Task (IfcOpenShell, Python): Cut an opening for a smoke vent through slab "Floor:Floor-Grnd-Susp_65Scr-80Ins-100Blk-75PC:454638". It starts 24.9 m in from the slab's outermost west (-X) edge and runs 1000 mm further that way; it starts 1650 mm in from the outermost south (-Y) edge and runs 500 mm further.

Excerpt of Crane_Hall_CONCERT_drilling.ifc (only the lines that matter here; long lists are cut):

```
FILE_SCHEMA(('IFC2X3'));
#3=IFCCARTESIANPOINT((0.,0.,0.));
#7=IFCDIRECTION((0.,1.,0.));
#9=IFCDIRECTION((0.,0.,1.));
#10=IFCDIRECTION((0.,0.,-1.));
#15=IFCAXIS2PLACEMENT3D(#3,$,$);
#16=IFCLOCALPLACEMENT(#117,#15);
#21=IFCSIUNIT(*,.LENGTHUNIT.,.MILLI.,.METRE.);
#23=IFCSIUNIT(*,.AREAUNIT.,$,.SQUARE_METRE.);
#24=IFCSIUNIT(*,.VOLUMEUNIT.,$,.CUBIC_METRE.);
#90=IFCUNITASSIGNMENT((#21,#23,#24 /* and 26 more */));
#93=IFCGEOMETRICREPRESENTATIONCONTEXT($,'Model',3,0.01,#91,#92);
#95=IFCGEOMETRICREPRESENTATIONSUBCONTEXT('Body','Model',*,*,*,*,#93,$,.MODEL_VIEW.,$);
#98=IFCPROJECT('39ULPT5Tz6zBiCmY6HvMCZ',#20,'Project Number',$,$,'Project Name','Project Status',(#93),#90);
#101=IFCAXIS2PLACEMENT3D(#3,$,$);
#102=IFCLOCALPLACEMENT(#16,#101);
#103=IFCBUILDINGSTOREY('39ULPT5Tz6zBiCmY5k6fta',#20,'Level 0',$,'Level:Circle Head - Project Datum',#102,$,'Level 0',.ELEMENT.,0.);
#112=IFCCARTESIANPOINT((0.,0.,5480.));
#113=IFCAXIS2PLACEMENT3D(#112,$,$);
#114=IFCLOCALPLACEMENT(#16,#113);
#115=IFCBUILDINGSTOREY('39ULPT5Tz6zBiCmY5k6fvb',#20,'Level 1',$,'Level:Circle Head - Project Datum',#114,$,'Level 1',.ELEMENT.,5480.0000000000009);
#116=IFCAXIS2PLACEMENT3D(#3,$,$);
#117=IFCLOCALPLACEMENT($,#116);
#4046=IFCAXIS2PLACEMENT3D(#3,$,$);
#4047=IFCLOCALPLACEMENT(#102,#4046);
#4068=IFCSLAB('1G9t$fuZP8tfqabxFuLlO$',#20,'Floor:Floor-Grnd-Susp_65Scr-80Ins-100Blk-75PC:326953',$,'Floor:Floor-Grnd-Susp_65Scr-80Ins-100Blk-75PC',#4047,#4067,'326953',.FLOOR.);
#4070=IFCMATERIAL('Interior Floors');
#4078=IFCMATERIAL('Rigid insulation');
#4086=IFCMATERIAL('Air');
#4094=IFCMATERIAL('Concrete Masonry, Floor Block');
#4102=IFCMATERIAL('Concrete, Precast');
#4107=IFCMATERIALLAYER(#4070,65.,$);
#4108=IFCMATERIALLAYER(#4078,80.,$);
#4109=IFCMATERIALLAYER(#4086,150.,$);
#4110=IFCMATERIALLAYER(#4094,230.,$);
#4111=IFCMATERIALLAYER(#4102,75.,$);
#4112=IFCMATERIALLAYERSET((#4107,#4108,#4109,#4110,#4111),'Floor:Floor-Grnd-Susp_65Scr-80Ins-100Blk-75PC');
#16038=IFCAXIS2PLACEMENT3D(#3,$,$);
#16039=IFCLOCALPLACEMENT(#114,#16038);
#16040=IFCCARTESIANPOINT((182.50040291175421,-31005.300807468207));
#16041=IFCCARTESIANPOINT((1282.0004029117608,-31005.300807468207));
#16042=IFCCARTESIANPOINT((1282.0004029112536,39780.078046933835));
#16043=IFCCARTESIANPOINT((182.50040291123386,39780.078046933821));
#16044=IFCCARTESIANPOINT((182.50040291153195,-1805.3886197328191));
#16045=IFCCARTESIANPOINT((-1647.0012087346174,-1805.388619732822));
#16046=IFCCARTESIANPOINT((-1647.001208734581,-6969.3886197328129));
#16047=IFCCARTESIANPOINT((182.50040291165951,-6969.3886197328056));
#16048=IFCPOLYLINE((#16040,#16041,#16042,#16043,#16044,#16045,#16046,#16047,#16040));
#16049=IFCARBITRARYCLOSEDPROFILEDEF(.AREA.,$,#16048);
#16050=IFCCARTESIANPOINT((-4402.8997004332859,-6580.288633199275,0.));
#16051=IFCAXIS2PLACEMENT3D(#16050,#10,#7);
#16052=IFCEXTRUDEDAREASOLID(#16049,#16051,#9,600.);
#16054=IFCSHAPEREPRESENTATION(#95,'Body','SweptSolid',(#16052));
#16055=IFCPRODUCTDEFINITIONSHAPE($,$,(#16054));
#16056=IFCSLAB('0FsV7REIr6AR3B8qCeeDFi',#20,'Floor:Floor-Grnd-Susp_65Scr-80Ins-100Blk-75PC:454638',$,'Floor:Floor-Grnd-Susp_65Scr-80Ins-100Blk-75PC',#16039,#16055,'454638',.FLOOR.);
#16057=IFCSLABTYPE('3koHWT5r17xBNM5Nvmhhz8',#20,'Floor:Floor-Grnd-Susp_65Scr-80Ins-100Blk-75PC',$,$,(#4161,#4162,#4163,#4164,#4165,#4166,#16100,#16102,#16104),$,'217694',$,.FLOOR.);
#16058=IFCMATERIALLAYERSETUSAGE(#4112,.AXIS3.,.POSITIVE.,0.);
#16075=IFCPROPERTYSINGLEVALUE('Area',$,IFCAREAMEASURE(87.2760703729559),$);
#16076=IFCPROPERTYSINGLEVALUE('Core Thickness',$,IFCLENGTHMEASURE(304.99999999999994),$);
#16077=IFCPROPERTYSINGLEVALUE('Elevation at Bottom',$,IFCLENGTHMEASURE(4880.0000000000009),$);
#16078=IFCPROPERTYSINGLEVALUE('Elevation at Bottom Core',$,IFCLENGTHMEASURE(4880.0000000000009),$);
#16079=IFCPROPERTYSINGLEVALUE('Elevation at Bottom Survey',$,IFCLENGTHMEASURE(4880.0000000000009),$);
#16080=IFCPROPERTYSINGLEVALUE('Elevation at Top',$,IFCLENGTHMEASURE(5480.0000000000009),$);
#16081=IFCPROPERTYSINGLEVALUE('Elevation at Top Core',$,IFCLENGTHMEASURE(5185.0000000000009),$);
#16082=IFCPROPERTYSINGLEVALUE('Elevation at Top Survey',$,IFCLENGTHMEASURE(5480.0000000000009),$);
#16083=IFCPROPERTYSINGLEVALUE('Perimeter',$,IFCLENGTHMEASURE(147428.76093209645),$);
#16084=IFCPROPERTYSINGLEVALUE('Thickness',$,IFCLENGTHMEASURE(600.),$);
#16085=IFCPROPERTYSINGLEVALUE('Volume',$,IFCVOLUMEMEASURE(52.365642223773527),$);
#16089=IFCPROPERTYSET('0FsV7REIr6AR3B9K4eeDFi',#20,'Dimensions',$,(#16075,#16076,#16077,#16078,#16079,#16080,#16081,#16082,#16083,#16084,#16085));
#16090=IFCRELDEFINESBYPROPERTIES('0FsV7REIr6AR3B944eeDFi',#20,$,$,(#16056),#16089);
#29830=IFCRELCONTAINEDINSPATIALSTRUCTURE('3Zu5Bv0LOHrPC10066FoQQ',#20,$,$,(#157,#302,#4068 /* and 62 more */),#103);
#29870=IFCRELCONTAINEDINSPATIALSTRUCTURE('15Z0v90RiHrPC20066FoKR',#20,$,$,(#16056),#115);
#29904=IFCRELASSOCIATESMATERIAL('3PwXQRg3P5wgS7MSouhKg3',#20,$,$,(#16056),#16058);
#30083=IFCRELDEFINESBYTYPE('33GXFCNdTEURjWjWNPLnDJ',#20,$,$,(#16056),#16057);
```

```python
import numpy as np
import ifcopenshell
import ifcopenshell.api.feature
import ifcopenshell.api.geometry
import ifcopenshell.api.pset
import ifcopenshell.api.root
import ifcopenshell.geom
import ifcopenshell.util.element
import ifcopenshell.util.placement
import ifcopenshell.util.representation
import ifcopenshell.util.shape
import ifcopenshell.util.unit

model = ifcopenshell.open("Crane_Hall_CONCERT_drilling.ifc")
unit_scale = ifcopenshell.util.unit.calculate_unit_scale(model)
area_scale = ifcopenshell.util.unit.calculate_unit_scale(model, "AREAUNIT")
volume_scale = ifcopenshell.util.unit.calculate_unit_scale(model, "VOLUMEUNIT")
settings = ifcopenshell.geom.settings()


def volume(element):
    """Net volume in cubic metres, openings subtracted."""
    shape = ifcopenshell.geom.create_shape(settings, element)
    return ifcopenshell.util.shape.get_volume(shape.geometry)


slab = model.by_guid("0FsV7REIr6AR3B8qCeeDFi")
before = volume(slab)

# Extent in the slab's own axes, in metres. The edges named are its -X and -Y sides.
slab_shape = ifcopenshell.geom.create_shape(settings, slab)
vertices = ifcopenshell.util.shape.get_vertices(slab_shape.geometry)
x_min, y_min, bottom = vertices.min(axis=0)
top = vertices[:, 2].max()

opening = ifcopenshell.api.root.create_entity(model, ifc_class="IfcOpeningElement", name="Smoke vent opening")
context = ifcopenshell.util.representation.get_context(model, "Model", "Body", "MODEL_VIEW")
width, depth = 1, 0.5
outline = [(0.0, 0.0), (width, 0.0), (width, depth), (0.0, depth), (0.0, 0.0)]
# Overshoot both faces by 50 mm so the cut is clean.
shape = ifcopenshell.api.geometry.add_slab_representation(
    model, context=context, depth=top - bottom + 0.1, polyline=outline
)
ifcopenshell.api.geometry.assign_representation(model, product=opening, representation=shape)

matrix = ifcopenshell.util.placement.get_local_placement(slab.ObjectPlacement)
matrix[:, 3] = matrix @ np.append(np.array([x_min + 24.9, y_min + 1.65, bottom - 0.05]) / unit_scale, 1.0)
ifcopenshell.api.geometry.edit_object_placement(model, product=opening, matrix=matrix, is_si=False)
ifcopenshell.api.feature.add_feature(model, feature=opening, element=slab)

after = volume(slab)

# Update the slab's stored quantities.
pset = model.by_id(ifcopenshell.util.element.get_pset(slab, "Dimensions", should_inherit=False)["id"])
ifcopenshell.api.pset.edit_pset(model, pset=pset, properties={
    "Area": model.create_entity("IfcAreaMeasure", after / (top - bottom) / area_scale),
    "Volume": model.create_entity("IfcVolumeMeasure", after / volume_scale),
})

print(f"slab volume {before:.3f} -> {after:.3f} m3")

model.write("Crane_Hall_CONCERT_drilling_rev.ifc")
```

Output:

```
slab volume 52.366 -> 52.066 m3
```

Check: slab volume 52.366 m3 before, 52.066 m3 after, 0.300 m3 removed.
